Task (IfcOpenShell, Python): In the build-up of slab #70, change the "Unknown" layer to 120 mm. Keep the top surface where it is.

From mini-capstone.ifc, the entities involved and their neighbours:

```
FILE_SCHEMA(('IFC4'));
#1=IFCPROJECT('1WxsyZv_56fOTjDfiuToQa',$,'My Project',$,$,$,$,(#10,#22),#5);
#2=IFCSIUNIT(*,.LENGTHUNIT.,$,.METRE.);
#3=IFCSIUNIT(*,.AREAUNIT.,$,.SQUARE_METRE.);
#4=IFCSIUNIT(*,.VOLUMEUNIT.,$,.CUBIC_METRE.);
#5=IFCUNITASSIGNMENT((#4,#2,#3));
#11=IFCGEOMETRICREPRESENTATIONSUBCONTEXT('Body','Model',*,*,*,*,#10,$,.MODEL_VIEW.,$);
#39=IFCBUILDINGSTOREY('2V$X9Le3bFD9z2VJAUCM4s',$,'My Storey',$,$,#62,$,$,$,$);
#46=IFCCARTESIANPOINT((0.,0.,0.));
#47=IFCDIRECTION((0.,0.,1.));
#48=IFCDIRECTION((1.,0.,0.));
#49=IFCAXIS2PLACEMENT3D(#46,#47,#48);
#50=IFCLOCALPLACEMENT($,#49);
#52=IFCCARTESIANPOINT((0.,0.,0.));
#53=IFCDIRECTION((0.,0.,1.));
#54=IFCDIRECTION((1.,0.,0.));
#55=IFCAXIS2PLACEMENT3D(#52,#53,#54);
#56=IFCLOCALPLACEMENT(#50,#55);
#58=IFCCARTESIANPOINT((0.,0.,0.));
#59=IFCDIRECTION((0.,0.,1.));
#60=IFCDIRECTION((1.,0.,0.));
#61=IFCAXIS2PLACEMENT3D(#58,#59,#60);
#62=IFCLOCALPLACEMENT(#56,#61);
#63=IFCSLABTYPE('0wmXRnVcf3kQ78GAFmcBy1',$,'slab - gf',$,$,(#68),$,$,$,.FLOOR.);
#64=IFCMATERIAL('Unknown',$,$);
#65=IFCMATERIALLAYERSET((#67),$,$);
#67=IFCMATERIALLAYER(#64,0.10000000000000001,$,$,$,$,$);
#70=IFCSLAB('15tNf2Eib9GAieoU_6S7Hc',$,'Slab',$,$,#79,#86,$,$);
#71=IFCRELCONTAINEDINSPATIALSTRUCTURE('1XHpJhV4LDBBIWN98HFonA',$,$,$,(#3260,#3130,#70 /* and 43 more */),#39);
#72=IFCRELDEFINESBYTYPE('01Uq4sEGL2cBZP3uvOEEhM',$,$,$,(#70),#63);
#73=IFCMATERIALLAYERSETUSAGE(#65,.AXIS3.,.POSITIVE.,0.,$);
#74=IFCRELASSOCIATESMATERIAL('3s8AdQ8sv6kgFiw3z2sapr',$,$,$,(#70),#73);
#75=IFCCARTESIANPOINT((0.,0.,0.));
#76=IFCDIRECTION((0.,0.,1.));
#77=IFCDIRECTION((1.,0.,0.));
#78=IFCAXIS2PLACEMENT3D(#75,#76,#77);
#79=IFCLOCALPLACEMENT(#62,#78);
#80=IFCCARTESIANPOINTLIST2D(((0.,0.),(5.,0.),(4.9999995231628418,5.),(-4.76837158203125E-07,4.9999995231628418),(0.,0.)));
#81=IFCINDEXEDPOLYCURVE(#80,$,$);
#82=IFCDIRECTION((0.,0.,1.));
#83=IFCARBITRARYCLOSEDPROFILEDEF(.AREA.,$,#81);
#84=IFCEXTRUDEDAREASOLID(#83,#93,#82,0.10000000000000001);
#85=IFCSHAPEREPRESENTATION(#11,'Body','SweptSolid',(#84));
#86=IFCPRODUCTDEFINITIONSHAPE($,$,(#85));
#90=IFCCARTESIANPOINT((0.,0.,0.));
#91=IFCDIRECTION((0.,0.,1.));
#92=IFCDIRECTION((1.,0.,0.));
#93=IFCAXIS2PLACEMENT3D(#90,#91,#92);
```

```python
import ifcopenshell
import ifcopenshell.util.element
import ifcopenshell.util.representation

model = ifcopenshell.open("mini-capstone.ifc")

layer_set = model.by_id(65)
layer = next(l for l in layer_set.MaterialLayers if l.Material and l.Material.Name == "Unknown")
change = 0.12 - layer.LayerThickness
layer.LayerThickness += change

# Geometry does not follow the layer set by itself.
slabs = [e for e in ifcopenshell.util.element.get_elements_by_material(model, layer_set) if e.is_a("IfcSlab")]
for slab in sorted(slabs, key=lambda e: e.id()):
    body = ifcopenshell.util.representation.get_representation(slab, "Model", "Body")
    solid = body.Items[0]
    old_depth = solid.Depth
    solid.Depth += change
    # Extruded upwards: lower the start of the extrusion so the top stays.
    x, y, z = solid.Position.Location.Coordinates
    solid.Position.Location = model.createIfcCartesianPoint((x, y, z - change))
    print(slab.id(), f"{old_depth:g} -> {solid.Depth:g}")

# The layers are counted up from the underside, which has moved.
for usage in {ifcopenshell.util.element.get_material(slab) for slab in slabs}:
    usage.OffsetFromReferenceLine -= change

model.write("mini-capstone_rev.ifc")
```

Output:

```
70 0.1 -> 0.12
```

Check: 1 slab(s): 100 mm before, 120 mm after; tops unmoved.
